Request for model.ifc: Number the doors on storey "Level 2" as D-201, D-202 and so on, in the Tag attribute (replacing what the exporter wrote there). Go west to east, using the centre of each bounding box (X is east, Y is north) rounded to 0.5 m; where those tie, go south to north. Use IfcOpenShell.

First a look at what the model holds.

```python
import ifcopenshell
import ifcopenshell.util.element
import ifcopenshell.util.placement

model = ifcopenshell.open("model.ifc")
print(model.schema)
storey = next(s for s in model.by_type("IfcBuildingStorey") if s.Name == "Level 2")
doors = [e for e in ifcopenshell.util.element.get_decomposition(storey) if e.is_a("IfcDoor")]
for e in sorted(doors, key=lambda e: e.id()):
    origin = ifcopenshell.util.placement.get_local_placement(e.ObjectPlacement)[:3, 3]
    print(e.id(), e.Tag, e.Name, origin.round(2) + 0.0, sep=" | ")
```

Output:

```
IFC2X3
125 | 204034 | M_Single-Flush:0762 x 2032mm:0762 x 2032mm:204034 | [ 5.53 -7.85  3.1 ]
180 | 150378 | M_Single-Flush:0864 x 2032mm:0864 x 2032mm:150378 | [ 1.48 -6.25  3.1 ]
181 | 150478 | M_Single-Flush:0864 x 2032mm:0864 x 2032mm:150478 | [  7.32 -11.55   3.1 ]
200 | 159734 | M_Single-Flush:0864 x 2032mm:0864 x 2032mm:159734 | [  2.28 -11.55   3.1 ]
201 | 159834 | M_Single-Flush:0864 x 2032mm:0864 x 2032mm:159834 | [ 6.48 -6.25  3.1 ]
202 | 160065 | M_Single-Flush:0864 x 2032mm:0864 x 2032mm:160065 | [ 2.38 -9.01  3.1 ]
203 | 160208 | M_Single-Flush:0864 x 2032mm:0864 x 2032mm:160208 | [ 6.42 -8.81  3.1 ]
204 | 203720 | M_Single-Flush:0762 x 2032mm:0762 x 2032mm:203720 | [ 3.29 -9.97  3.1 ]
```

```python
import ifcopenshell
import ifcopenshell.geom
import ifcopenshell.util.element
import ifcopenshell.util.shape

model = ifcopenshell.open("model.ifc")
settings = ifcopenshell.geom.settings()
settings.set("use-world-coords", True)


def centre(element):
    shape = ifcopenshell.geom.create_shape(settings, element)
    return ifcopenshell.util.shape.get_bbox_centroid(shape.geometry)


storey = next(s for s in model.by_type("IfcBuildingStorey") if s.Name == "Level 2")
doors = [e for e in ifcopenshell.util.element.get_decomposition(storey) if e.is_a("IfcDoor")]

# Insertion points can sit at a corner or the storey origin, so sort by the geometry (in metres).
centres = {e: centre(e) for e in doors}
doors.sort(key=lambda e: (round(centres[e][0] / 0.5), centres[e][1]))

for i, e in enumerate(doors, start=1):
    number = f"D-2{i:02d}"
    e.Tag = number
    print(e.id(), number)

model.write("model_edited.ifc")
```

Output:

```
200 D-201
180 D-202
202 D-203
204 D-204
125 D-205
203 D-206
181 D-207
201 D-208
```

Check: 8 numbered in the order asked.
